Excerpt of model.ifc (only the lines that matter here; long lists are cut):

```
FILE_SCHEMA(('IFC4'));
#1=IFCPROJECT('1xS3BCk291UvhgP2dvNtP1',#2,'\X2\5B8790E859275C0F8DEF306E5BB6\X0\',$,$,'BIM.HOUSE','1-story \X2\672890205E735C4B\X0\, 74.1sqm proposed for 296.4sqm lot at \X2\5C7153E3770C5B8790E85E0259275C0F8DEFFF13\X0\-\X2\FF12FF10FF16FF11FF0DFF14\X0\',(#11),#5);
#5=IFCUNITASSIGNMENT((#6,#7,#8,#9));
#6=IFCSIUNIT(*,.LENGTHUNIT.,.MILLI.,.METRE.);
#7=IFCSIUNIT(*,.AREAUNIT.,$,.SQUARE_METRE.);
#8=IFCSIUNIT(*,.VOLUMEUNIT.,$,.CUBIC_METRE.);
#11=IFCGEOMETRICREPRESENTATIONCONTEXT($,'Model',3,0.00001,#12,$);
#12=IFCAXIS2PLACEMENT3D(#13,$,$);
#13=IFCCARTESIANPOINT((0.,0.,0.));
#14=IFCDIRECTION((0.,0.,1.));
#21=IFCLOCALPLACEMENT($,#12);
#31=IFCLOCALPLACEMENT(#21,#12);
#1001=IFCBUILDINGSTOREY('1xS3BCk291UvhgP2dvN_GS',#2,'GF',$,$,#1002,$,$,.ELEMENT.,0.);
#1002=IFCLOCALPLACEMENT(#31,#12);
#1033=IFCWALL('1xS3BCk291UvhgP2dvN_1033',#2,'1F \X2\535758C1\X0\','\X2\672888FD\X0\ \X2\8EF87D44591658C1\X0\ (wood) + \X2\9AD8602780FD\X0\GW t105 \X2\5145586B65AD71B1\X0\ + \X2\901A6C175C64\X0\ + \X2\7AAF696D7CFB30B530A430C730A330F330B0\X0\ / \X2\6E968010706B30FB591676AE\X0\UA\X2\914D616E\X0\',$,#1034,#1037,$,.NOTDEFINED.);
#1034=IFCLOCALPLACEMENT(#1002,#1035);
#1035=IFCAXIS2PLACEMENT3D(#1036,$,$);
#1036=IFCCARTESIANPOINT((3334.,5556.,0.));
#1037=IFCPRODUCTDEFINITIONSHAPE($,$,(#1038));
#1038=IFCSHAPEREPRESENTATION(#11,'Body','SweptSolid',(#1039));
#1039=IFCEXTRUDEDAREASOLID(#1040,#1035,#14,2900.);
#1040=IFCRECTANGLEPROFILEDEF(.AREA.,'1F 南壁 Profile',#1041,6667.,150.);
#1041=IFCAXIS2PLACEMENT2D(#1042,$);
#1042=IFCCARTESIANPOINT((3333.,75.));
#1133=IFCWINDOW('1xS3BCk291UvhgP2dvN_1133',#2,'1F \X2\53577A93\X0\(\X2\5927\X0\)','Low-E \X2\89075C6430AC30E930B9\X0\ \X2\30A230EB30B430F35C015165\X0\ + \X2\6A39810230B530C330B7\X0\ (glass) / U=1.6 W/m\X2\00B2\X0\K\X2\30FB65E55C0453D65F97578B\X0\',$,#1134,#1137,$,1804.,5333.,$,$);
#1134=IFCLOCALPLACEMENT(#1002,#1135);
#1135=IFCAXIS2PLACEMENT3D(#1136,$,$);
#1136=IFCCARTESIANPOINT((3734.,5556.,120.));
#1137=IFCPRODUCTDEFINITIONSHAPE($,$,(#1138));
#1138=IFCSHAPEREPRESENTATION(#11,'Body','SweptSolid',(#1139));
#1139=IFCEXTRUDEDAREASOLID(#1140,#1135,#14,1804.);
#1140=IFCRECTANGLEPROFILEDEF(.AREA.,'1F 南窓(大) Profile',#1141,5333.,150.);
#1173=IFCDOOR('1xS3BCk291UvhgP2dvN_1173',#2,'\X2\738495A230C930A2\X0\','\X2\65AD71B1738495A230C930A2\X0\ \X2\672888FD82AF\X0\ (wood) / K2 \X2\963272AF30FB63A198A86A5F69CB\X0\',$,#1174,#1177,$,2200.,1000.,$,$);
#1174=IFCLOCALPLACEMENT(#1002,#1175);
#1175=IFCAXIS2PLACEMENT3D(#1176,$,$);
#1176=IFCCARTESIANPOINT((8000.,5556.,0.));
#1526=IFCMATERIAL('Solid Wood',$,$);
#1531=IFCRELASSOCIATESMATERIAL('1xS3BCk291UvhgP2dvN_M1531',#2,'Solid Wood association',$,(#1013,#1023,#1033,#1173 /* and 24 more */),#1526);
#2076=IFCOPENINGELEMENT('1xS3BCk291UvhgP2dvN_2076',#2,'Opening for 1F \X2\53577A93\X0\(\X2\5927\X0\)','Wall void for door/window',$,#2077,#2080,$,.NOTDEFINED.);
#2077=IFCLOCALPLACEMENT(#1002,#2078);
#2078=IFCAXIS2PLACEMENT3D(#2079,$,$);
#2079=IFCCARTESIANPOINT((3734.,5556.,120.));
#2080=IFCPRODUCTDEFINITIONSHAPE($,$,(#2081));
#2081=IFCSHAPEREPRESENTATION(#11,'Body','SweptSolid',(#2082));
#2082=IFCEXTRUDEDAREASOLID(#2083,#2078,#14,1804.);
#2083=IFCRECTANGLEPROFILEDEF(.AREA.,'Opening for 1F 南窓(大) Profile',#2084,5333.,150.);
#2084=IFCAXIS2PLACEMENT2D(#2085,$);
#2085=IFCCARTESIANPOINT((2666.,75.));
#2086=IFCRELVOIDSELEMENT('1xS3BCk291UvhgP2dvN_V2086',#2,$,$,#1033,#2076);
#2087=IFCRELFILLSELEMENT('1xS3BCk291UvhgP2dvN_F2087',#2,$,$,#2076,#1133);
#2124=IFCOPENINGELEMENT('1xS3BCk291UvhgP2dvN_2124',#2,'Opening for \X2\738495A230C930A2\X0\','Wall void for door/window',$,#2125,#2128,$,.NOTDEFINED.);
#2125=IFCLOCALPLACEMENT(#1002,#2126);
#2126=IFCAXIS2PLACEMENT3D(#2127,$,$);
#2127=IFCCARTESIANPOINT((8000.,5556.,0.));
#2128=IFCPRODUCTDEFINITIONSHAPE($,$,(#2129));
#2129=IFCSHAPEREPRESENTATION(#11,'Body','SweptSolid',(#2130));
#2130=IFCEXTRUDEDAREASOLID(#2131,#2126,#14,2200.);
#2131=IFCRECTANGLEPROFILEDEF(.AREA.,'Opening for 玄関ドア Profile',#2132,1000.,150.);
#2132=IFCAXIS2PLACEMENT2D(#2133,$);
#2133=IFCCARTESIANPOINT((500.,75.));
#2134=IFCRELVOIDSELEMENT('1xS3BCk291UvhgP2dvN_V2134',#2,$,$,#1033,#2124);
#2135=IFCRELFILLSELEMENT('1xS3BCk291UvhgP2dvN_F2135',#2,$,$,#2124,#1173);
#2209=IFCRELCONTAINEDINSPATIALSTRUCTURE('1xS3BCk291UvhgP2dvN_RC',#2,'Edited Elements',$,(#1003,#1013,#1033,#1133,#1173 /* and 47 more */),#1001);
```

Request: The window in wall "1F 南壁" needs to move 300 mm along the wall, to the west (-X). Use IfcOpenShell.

```python
import ifcopenshell
import ifcopenshell.api.geometry
import ifcopenshell.util.placement
import ifcopenshell.util.unit

model = ifcopenshell.open("model.ifc")
unit_scale = ifcopenshell.util.unit.calculate_unit_scale(model)

window = model.by_guid("1xS3BCk291UvhgP2dvN_1133")
opening = window.FillsVoids[0].RelatingOpeningElement
wall = opening.VoidsElements[0].RelatingBuildingElement

wall_matrix = ifcopenshell.util.placement.get_local_placement(wall.ObjectPlacement)
shift = wall_matrix[:3, 0] * -0.3 / unit_scale
before = ifcopenshell.util.placement.get_local_placement(window.ObjectPlacement)[:3, 3].copy()

# The window is not placed relative to its opening, so move both.
for product in (opening, window):
    matrix = ifcopenshell.util.placement.get_local_placement(product.ObjectPlacement)
    matrix[:3, 3] += shift
    ifcopenshell.api.geometry.edit_object_placement(model, product=product, matrix=matrix, is_si=False)

after = ifcopenshell.util.placement.get_local_placement(window.ObjectPlacement)[:3, 3]
print("window moved by", (after - before).round(3) + 0.0)

model.write("model_edited.ifc")
```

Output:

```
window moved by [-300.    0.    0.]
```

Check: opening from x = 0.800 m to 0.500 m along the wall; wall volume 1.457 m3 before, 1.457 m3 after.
